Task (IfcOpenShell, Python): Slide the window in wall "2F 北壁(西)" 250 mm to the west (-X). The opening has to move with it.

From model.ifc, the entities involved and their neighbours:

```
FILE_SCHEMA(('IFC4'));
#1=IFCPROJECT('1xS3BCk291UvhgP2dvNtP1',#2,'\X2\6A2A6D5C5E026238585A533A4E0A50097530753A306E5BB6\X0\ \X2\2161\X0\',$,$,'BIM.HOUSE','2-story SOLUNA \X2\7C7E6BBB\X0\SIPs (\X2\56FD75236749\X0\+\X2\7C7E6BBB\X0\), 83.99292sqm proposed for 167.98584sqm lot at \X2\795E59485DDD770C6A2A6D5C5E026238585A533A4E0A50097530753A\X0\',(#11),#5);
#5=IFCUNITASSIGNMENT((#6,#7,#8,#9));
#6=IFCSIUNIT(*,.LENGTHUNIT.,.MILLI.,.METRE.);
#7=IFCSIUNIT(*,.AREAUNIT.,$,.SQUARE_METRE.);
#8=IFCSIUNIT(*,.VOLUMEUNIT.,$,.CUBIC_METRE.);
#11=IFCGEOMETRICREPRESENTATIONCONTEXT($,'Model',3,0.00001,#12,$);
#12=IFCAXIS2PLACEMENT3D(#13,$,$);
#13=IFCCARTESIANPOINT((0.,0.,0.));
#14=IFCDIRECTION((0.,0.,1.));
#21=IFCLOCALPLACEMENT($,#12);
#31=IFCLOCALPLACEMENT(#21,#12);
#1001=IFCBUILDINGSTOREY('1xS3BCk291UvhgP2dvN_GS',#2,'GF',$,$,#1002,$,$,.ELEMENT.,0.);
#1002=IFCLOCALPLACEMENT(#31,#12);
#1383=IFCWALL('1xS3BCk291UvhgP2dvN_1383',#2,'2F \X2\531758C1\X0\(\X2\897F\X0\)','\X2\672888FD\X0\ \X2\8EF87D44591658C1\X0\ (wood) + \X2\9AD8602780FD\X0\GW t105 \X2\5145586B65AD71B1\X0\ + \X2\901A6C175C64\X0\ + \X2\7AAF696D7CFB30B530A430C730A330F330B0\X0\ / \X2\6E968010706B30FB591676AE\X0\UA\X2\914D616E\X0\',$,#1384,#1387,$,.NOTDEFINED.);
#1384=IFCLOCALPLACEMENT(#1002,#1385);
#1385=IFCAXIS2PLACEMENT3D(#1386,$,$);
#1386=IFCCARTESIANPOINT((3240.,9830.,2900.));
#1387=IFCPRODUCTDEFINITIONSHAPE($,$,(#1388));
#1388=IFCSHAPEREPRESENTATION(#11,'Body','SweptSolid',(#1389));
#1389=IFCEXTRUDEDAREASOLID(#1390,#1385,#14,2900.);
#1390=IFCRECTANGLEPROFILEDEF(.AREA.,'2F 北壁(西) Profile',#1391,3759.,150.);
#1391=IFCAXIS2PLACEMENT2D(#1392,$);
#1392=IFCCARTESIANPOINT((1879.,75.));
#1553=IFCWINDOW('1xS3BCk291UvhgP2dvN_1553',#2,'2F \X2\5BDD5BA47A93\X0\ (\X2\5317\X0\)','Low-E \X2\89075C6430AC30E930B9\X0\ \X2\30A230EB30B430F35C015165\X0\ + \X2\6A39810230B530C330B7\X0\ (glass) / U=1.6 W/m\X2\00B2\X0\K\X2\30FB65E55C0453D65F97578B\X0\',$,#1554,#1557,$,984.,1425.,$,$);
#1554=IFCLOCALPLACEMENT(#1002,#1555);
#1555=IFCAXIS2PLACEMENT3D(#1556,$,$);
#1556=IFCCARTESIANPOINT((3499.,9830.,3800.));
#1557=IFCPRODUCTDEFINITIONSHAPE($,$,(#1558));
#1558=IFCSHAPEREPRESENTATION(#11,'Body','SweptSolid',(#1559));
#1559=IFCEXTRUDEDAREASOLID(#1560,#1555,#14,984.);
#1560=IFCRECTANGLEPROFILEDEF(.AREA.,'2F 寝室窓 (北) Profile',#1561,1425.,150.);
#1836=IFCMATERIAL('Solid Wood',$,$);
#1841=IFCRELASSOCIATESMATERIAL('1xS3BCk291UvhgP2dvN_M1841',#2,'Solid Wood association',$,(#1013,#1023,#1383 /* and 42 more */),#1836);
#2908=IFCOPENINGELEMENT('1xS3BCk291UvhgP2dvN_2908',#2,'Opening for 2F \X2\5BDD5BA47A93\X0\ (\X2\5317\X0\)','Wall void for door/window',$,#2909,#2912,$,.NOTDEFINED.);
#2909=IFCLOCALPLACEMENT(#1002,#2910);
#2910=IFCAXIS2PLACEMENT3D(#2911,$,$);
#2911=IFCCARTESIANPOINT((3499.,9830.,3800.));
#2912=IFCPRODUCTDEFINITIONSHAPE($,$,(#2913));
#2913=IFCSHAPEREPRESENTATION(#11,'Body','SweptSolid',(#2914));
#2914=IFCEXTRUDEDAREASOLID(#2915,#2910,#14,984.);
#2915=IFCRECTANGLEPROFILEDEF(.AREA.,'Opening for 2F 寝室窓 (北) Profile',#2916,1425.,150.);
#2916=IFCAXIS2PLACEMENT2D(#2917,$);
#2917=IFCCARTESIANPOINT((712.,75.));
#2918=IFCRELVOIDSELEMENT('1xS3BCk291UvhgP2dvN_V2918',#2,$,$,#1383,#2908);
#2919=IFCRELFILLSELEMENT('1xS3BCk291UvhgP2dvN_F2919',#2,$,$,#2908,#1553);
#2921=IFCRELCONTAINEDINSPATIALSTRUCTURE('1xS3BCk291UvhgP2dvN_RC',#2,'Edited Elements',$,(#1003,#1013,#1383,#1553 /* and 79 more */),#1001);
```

```python
import ifcopenshell
import ifcopenshell.api.geometry
import ifcopenshell.util.placement

model = ifcopenshell.open("model.ifc")

window = model.by_id(1553)
opening = window.FillsVoids[0].RelatingOpeningElement
wall = opening.VoidsElements[0].RelatingBuildingElement

wall_matrix = ifcopenshell.util.placement.get_local_placement(wall.ObjectPlacement)
shift = wall_matrix[:3, 0] * -250.0
before = ifcopenshell.util.placement.get_local_placement(window.ObjectPlacement)[:3, 3].copy()

# The window is not placed relative to its opening, so move both.
for product in (opening, window):
    matrix = ifcopenshell.util.placement.get_local_placement(product.ObjectPlacement)
    matrix[:3, 3] += shift
    ifcopenshell.api.geometry.edit_object_placement(model, product=product, matrix=matrix, is_si=False)

after = ifcopenshell.util.placement.get_local_placement(window.ObjectPlacement)[:3, 3]
print("window moved by", (after - before).round(3) + 0.0)

model.write("model_v2.ifc")
```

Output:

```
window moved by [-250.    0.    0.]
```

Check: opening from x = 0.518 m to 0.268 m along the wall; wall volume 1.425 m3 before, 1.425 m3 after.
